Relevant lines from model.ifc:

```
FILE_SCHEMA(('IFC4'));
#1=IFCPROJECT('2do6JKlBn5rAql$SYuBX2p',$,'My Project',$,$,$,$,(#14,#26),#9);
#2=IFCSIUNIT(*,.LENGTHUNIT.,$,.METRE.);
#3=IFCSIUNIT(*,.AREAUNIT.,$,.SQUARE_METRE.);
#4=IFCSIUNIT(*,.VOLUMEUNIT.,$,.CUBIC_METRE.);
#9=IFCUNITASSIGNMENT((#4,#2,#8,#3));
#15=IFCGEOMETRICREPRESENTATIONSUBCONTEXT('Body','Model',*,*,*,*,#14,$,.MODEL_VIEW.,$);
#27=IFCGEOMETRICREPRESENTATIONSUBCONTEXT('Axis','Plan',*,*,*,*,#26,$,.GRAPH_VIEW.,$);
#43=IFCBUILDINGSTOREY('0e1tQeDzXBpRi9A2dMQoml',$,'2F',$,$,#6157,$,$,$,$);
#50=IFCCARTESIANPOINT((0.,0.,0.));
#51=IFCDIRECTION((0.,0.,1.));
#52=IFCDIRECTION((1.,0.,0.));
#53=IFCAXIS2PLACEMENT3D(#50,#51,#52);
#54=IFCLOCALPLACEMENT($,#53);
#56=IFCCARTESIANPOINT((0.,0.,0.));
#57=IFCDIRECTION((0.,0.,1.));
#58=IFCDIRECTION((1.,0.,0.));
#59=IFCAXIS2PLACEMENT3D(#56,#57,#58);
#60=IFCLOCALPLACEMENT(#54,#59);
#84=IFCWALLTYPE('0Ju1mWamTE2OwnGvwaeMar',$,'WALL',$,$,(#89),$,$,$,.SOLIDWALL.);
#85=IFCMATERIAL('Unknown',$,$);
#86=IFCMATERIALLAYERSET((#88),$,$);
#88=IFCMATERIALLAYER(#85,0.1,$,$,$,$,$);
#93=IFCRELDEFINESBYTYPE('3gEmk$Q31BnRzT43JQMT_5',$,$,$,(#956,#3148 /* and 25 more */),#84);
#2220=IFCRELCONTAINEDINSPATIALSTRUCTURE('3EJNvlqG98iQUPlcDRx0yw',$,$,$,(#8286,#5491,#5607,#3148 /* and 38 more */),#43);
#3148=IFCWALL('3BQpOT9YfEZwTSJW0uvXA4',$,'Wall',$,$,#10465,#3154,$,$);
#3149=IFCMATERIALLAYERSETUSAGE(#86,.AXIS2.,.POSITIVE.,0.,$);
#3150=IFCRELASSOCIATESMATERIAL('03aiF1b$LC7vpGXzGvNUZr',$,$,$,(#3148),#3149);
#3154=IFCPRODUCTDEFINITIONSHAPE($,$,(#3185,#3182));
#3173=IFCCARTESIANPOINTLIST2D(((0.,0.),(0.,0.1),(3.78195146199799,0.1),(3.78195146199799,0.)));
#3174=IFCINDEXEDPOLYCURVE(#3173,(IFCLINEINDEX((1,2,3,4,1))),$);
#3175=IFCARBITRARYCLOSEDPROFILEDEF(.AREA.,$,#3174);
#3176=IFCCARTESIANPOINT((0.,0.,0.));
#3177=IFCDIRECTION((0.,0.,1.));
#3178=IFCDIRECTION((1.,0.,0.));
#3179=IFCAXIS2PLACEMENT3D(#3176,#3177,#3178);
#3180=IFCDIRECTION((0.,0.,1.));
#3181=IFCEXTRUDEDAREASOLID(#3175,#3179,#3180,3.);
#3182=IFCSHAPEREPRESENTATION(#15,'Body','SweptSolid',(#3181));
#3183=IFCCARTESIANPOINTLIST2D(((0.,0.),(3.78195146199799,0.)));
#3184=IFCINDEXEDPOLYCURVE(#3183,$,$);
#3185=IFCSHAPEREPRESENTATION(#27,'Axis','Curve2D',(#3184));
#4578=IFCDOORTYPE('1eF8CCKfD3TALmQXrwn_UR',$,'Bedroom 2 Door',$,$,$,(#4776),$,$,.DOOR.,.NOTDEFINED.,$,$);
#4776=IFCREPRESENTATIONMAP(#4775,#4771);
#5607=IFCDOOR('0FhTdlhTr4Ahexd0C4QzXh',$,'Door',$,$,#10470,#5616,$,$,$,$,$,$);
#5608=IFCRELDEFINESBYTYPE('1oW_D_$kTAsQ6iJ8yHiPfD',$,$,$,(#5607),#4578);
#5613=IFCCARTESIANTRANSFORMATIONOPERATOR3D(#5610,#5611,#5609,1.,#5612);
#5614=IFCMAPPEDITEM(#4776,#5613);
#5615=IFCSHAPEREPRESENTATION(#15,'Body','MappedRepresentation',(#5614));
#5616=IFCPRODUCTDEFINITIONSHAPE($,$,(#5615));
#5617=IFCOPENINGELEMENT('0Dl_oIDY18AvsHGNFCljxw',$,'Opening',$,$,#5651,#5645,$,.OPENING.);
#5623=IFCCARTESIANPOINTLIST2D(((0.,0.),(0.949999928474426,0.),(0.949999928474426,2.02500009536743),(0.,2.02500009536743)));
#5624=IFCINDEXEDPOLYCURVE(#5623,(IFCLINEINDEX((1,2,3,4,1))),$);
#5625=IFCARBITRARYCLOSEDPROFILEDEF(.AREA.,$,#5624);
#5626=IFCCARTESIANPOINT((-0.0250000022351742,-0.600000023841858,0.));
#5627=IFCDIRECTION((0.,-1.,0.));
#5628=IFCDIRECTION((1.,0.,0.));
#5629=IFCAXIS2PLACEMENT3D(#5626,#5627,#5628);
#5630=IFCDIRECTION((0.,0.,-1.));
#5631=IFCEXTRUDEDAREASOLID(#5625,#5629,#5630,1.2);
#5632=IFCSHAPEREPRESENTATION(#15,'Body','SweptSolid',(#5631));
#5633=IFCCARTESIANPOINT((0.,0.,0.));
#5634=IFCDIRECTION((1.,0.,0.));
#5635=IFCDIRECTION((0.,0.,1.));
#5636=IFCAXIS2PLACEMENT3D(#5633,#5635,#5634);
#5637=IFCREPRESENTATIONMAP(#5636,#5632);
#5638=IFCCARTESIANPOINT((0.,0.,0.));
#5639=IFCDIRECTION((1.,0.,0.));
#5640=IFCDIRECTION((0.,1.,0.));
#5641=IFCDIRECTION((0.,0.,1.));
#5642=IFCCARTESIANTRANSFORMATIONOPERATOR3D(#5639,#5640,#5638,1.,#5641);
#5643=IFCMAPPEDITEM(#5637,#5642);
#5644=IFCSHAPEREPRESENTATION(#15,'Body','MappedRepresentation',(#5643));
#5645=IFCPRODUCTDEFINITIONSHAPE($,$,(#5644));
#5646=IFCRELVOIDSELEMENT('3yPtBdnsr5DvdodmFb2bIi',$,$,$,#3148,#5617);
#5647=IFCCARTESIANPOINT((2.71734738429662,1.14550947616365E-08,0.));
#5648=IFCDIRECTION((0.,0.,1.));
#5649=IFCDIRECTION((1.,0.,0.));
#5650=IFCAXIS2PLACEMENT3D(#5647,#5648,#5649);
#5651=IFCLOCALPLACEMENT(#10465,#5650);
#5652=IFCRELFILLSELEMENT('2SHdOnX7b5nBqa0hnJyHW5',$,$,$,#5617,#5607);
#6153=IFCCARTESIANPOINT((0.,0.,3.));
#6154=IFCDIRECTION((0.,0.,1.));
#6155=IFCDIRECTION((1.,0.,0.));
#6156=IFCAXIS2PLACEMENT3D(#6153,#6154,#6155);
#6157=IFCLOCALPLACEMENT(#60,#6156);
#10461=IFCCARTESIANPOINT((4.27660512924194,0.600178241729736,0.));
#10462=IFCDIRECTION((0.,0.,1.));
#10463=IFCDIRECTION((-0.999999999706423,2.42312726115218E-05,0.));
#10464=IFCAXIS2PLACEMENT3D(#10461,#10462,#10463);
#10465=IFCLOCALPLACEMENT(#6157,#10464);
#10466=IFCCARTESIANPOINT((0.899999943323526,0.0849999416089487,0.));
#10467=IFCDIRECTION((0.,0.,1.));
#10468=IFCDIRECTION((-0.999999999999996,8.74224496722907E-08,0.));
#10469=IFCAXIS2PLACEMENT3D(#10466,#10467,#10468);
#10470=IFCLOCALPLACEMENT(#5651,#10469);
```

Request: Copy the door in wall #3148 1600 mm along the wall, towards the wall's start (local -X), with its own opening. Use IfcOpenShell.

```python
import ifcopenshell
import ifcopenshell.api.feature
import ifcopenshell.api.geometry
import ifcopenshell.api.root
import ifcopenshell.geom
import ifcopenshell.util.element
import ifcopenshell.util.placement
import ifcopenshell.util.shape
import ifcopenshell.util.unit

model = ifcopenshell.open("model.ifc")
unit_scale = ifcopenshell.util.unit.calculate_unit_scale(model)
settings = ifcopenshell.geom.settings()


def volume(element):
    """Net volume in cubic metres, openings subtracted."""
    shape = ifcopenshell.geom.create_shape(settings, element)
    return ifcopenshell.util.shape.get_volume(shape.geometry)


door = model.by_id(5607)
opening = door.FillsVoids[0].RelatingOpeningElement
wall = opening.VoidsElements[0].RelatingBuildingElement
before = volume(wall)
shift = ifcopenshell.util.placement.get_local_placement(wall.ObjectPlacement)[:3, 0] * -1.6 / unit_scale

# copy_class copies the void relationship, type, container and properties, but no geometry.
new_opening = ifcopenshell.api.root.copy_class(model, product=opening)
new_opening.Representation = ifcopenshell.util.element.copy_deep(
    model, opening.Representation, exclude=["IfcGeometricRepresentationContext", "IfcRepresentationMap"]
)
new_door = ifcopenshell.api.root.copy_class(model, product=door)
new_door.Representation = ifcopenshell.util.element.copy_deep(
    model, door.Representation, exclude=["IfcGeometricRepresentationContext", "IfcRepresentationMap"]
)
ifcopenshell.api.feature.add_filling(model, opening=new_opening, element=new_door)

for old, new in ((opening, new_opening), (door, new_door)):
    matrix = ifcopenshell.util.placement.get_local_placement(old.ObjectPlacement)
    matrix[:3, 3] += shift
    ifcopenshell.api.geometry.edit_object_placement(model, product=new, matrix=matrix, is_si=False)

after = volume(wall)

print(f"wall volume {before:.3f} -> {after:.3f} m3")

model.write("model_edited.ifc")
```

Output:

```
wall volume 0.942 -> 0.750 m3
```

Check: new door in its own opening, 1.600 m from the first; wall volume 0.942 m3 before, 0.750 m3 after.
